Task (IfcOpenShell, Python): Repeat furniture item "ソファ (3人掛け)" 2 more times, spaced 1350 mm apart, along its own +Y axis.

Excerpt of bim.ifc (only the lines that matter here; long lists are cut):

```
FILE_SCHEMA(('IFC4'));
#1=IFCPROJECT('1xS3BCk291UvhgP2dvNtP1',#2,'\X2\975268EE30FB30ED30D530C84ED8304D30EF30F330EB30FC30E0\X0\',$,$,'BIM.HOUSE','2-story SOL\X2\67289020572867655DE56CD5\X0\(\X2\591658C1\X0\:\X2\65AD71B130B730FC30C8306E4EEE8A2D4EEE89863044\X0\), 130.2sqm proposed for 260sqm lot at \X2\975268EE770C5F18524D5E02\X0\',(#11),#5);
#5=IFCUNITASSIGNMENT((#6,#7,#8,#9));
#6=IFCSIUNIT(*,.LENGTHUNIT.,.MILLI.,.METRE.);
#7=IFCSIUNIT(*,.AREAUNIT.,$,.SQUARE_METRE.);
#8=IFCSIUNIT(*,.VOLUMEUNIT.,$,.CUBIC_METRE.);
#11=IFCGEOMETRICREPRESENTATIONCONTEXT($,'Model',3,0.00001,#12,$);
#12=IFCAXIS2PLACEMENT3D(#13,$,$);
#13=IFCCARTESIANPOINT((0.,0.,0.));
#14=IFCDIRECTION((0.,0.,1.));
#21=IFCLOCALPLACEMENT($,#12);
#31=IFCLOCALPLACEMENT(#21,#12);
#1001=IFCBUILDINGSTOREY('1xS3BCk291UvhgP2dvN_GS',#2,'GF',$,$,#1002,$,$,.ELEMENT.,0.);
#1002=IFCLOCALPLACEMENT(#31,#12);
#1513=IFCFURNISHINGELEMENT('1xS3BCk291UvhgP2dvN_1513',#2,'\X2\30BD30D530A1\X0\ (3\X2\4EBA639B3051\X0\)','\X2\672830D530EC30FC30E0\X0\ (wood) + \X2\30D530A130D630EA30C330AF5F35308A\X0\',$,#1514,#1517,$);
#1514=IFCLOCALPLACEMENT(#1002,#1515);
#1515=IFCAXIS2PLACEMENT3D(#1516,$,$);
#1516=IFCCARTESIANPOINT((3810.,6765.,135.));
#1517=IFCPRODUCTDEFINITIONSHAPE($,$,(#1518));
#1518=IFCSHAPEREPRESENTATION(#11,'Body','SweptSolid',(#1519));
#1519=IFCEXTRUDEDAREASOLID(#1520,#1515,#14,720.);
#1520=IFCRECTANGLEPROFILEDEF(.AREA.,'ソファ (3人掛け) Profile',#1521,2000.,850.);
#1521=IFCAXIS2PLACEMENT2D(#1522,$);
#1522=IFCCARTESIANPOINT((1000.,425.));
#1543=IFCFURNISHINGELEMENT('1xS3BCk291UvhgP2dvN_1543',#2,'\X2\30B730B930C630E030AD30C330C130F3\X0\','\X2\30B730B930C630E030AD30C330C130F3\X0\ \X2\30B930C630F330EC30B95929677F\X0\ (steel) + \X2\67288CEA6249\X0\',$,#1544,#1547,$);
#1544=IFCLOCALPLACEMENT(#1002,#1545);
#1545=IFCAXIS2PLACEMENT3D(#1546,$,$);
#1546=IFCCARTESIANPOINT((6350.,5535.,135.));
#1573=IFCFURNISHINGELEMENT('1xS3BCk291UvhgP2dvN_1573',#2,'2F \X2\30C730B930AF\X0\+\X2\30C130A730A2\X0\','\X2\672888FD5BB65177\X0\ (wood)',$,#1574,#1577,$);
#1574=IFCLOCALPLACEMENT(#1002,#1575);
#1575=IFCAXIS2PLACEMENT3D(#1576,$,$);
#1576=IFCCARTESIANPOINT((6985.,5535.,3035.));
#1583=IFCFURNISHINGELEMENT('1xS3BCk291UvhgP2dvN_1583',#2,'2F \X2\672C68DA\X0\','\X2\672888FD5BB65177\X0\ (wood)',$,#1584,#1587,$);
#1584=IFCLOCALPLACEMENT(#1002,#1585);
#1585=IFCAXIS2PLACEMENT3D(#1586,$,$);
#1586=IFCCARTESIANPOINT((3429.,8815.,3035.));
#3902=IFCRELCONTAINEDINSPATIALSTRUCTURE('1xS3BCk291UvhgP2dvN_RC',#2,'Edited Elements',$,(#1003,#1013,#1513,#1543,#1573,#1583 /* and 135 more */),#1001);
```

```python
import ifcopenshell
import ifcopenshell.api.geometry
import ifcopenshell.api.root
import ifcopenshell.util.element
import ifcopenshell.util.placement
import ifcopenshell.util.unit

model = ifcopenshell.open("bim.ifc")
unit_scale = ifcopenshell.util.unit.calculate_unit_scale(model)


def reuse_history(source, copy):
    """copy_class also copies each property set's owner history, people and application; keep the originals."""
    for rel in copy.IsDefinedBy:
        if rel.is_a("IfcRelDefinesByProperties") and (history := rel.RelatingPropertyDefinition.OwnerHistory):
            rel.RelatingPropertyDefinition.OwnerHistory = source.OwnerHistory
            ifcopenshell.util.element.remove_deep2(model, history)


source = model.by_guid("1xS3BCk291UvhgP2dvN_1513")
base = ifcopenshell.util.placement.get_local_placement(source.ObjectPlacement)
step = base[:3, 1] * 1.35 / unit_scale

for i in range(1, 3):
    copy = ifcopenshell.api.root.copy_class(model, product=source)
    copy.Representation = ifcopenshell.util.element.copy_deep(
        model, source.Representation, exclude=["IfcGeometricRepresentationContext", "IfcRepresentationMap"]
    )
    reuse_history(source, copy)
    matrix = base.copy()
    matrix[:3, 3] += i * step
    print("added at", matrix[:3, 3].round(3) + 0.0)
    ifcopenshell.api.geometry.edit_object_placement(model, product=copy, matrix=matrix, is_si=False)

model.write("bim_edited.ifc")
```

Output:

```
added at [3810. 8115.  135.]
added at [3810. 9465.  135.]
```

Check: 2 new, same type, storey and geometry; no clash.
